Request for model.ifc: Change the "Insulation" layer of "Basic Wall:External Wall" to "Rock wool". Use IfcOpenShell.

First a look at what the model holds.

```python
import ifcopenshell
import ifcopenshell.util.element

model = ifcopenshell.open("model.ifc")
print(model.schema)
for layer_set in model.by_type("IfcMaterialLayerSet"):
    if layer_set.LayerSetName == "Basic Wall:External Wall":
        for layer in layer_set.MaterialLayers:
            print(layer.id(), layer.Material and layer.Material.Name, layer.LayerThickness, sep=" | ")
        print(len(ifcopenshell.util.element.get_elements_by_material(model, layer_set)), "elements and types use it")
print(sorted(m.Name for m in model.by_type("IfcMaterial") if m.Name)[:60])
```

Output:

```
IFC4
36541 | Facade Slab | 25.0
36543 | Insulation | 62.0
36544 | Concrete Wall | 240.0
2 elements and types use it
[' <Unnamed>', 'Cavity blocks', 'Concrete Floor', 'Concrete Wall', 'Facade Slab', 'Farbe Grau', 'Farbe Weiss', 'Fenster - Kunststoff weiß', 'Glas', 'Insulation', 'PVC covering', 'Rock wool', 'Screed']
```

```python
import ifcopenshell
import ifcopenshell.api.material

model = ifcopenshell.open("model.ifc")

layer_set = next(s for s in model.by_type("IfcMaterialLayerSet") if s.LayerSetName == "Basic Wall:External Wall")
layer = next(l for l in layer_set.MaterialLayers if l.Material and l.Material.Name == "Insulation")
material = next(m for m in model.by_type("IfcMaterial") if m.Name == "Rock wool")

# Point this one layer at the other material; renaming the old one would change it everywhere.
ifcopenshell.api.material.edit_layer(model, layer=layer, attributes={}, material=material)

print([l.Material.Name if l.Material else None for l in layer_set.MaterialLayers])

model.write("model_v2.ifc")
```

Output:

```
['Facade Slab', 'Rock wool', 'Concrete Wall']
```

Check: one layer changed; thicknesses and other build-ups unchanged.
